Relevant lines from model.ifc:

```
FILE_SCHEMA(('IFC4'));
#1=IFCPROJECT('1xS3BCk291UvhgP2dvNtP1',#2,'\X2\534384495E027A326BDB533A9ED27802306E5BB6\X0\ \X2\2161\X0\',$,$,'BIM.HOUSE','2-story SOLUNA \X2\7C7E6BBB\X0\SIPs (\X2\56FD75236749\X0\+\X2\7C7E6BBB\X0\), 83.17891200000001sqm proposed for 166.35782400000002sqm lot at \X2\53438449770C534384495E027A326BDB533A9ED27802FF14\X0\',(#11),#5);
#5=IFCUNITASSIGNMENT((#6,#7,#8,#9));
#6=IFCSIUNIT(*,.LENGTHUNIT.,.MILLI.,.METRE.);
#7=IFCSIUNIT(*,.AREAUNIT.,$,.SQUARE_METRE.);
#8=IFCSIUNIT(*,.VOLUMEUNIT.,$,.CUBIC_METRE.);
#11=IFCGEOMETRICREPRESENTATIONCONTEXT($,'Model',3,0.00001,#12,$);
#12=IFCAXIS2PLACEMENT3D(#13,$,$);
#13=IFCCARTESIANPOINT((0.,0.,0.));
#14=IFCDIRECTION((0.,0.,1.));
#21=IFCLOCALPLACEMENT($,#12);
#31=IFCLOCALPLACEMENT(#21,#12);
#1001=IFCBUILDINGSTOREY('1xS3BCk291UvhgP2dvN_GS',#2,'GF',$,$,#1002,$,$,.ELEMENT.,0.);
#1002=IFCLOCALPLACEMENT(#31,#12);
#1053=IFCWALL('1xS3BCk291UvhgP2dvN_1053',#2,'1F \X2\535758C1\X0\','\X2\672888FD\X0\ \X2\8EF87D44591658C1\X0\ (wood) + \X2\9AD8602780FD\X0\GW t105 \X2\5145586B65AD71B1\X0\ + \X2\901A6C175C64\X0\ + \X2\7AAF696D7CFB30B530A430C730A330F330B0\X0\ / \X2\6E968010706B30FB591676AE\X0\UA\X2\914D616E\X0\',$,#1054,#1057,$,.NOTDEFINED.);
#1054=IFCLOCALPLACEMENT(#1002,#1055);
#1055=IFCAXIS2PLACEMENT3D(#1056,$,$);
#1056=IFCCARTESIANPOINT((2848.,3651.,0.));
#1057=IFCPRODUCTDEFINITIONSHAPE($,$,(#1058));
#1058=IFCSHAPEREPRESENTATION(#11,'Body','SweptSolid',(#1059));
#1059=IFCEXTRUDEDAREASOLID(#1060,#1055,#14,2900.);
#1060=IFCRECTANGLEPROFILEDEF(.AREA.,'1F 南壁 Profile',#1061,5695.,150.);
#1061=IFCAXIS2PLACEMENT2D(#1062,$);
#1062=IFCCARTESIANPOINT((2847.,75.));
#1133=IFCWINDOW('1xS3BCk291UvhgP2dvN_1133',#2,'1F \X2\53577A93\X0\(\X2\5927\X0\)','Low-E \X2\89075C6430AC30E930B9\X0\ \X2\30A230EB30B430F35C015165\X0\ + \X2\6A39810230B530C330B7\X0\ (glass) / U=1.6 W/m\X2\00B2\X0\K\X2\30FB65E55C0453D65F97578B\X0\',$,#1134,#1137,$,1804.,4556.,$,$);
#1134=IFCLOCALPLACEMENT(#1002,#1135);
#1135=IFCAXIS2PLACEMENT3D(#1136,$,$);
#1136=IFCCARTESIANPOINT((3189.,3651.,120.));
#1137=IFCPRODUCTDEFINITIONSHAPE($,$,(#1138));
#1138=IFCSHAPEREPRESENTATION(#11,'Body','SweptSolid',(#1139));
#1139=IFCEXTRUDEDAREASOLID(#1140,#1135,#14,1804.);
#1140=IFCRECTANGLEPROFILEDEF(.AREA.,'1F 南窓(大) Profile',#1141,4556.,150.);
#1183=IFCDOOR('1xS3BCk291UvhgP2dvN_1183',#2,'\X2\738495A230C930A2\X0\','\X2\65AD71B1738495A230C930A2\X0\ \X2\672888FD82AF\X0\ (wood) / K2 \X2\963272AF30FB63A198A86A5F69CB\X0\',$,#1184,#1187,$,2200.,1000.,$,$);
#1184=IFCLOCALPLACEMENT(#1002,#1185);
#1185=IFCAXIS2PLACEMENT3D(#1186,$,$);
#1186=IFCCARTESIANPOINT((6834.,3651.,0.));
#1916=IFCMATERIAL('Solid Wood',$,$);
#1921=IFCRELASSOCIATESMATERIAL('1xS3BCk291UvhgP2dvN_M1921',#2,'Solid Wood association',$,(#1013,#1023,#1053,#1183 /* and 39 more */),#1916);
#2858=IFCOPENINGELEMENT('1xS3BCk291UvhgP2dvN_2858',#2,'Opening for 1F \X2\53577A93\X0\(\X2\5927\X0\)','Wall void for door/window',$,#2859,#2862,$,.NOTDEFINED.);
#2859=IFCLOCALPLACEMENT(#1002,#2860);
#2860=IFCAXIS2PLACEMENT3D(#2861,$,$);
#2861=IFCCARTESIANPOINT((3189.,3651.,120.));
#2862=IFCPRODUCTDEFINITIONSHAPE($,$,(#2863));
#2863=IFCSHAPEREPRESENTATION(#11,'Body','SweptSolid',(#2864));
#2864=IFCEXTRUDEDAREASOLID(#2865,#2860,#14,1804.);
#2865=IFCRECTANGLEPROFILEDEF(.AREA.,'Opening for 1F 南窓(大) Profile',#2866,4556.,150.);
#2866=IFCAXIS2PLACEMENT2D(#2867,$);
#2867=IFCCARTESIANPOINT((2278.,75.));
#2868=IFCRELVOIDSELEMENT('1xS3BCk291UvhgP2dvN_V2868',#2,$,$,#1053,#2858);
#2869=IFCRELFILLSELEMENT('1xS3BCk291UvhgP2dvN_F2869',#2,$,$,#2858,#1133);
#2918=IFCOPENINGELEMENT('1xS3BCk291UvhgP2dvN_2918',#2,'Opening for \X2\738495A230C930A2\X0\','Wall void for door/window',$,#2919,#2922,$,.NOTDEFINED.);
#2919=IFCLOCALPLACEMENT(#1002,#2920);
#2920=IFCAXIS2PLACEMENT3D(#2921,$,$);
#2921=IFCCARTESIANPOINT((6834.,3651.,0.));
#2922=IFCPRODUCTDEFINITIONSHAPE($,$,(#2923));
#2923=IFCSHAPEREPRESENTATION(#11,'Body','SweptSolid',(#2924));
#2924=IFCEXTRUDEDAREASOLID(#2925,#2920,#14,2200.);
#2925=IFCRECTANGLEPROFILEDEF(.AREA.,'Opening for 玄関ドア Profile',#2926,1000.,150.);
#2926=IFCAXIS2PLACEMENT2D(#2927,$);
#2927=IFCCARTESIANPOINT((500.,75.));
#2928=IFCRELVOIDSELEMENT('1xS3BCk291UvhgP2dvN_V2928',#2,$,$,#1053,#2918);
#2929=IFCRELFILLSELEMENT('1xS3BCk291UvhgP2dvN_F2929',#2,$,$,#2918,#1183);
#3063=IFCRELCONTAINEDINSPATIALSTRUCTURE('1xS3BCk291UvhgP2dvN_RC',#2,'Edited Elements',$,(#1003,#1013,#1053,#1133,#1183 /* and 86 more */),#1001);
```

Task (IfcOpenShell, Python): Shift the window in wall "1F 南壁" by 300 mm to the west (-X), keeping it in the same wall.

```python
import ifcopenshell
import ifcopenshell.api.geometry
import ifcopenshell.util.placement

model = ifcopenshell.open("model.ifc")

window = model.by_guid("1xS3BCk291UvhgP2dvN_1133")
opening = window.FillsVoids[0].RelatingOpeningElement
wall = opening.VoidsElements[0].RelatingBuildingElement

wall_matrix = ifcopenshell.util.placement.get_local_placement(wall.ObjectPlacement)
shift = wall_matrix[:3, 0] * -300.0
before = ifcopenshell.util.placement.get_local_placement(window.ObjectPlacement)[:3, 3].copy()

# The window is not placed relative to its opening, so move both.
for product in (opening, window):
    matrix = ifcopenshell.util.placement.get_local_placement(product.ObjectPlacement)
    matrix[:3, 3] += shift
    ifcopenshell.api.geometry.edit_object_placement(model, product=product, matrix=matrix, is_si=False)

after = ifcopenshell.util.placement.get_local_placement(window.ObjectPlacement)[:3, 3]
print("window moved by", (after - before).round(3) + 0.0)

model.write("model_v2.ifc")
```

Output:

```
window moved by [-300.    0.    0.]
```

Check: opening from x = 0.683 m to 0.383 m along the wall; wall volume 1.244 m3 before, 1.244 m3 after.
